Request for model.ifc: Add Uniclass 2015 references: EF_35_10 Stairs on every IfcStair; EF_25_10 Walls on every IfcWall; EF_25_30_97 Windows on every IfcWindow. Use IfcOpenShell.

First a look at what the model holds.

```python
import ifcopenshell

model = ifcopenshell.open("model.ifc")
print(model.schema)
print("classifications:", [c.Name for c in model.by_type("IfcClassification")])
for ifc_class in ("IfcDoor", "IfcRoof", "IfcStair", "IfcWall", "IfcWindow"):
    print(ifc_class, len(model.by_type(ifc_class)))
```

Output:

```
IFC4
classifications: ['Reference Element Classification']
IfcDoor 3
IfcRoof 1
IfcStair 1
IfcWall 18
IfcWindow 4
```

```python
import ifcopenshell
import ifcopenshell.api.classification

model = ifcopenshell.open("model.ifc")

system = ifcopenshell.api.classification.add_classification(model, classification="Uniclass 2015")

codes = {
    "IfcStair": ("EF_35_10", "Stairs"),
    "IfcWall": ("EF_25_10", "Walls"),
    "IfcWindow": ("EF_25_30_97", "Windows"),
}
for ifc_class, (code, name) in codes.items():
    products = model.by_type(ifc_class)
    ifcopenshell.api.classification.add_reference(
        model, products=products, classification=system, identification=code, name=name
    )
    print(code, len(products))

model.write("model-out.ifc")
```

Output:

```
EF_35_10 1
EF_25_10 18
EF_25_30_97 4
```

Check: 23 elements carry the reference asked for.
